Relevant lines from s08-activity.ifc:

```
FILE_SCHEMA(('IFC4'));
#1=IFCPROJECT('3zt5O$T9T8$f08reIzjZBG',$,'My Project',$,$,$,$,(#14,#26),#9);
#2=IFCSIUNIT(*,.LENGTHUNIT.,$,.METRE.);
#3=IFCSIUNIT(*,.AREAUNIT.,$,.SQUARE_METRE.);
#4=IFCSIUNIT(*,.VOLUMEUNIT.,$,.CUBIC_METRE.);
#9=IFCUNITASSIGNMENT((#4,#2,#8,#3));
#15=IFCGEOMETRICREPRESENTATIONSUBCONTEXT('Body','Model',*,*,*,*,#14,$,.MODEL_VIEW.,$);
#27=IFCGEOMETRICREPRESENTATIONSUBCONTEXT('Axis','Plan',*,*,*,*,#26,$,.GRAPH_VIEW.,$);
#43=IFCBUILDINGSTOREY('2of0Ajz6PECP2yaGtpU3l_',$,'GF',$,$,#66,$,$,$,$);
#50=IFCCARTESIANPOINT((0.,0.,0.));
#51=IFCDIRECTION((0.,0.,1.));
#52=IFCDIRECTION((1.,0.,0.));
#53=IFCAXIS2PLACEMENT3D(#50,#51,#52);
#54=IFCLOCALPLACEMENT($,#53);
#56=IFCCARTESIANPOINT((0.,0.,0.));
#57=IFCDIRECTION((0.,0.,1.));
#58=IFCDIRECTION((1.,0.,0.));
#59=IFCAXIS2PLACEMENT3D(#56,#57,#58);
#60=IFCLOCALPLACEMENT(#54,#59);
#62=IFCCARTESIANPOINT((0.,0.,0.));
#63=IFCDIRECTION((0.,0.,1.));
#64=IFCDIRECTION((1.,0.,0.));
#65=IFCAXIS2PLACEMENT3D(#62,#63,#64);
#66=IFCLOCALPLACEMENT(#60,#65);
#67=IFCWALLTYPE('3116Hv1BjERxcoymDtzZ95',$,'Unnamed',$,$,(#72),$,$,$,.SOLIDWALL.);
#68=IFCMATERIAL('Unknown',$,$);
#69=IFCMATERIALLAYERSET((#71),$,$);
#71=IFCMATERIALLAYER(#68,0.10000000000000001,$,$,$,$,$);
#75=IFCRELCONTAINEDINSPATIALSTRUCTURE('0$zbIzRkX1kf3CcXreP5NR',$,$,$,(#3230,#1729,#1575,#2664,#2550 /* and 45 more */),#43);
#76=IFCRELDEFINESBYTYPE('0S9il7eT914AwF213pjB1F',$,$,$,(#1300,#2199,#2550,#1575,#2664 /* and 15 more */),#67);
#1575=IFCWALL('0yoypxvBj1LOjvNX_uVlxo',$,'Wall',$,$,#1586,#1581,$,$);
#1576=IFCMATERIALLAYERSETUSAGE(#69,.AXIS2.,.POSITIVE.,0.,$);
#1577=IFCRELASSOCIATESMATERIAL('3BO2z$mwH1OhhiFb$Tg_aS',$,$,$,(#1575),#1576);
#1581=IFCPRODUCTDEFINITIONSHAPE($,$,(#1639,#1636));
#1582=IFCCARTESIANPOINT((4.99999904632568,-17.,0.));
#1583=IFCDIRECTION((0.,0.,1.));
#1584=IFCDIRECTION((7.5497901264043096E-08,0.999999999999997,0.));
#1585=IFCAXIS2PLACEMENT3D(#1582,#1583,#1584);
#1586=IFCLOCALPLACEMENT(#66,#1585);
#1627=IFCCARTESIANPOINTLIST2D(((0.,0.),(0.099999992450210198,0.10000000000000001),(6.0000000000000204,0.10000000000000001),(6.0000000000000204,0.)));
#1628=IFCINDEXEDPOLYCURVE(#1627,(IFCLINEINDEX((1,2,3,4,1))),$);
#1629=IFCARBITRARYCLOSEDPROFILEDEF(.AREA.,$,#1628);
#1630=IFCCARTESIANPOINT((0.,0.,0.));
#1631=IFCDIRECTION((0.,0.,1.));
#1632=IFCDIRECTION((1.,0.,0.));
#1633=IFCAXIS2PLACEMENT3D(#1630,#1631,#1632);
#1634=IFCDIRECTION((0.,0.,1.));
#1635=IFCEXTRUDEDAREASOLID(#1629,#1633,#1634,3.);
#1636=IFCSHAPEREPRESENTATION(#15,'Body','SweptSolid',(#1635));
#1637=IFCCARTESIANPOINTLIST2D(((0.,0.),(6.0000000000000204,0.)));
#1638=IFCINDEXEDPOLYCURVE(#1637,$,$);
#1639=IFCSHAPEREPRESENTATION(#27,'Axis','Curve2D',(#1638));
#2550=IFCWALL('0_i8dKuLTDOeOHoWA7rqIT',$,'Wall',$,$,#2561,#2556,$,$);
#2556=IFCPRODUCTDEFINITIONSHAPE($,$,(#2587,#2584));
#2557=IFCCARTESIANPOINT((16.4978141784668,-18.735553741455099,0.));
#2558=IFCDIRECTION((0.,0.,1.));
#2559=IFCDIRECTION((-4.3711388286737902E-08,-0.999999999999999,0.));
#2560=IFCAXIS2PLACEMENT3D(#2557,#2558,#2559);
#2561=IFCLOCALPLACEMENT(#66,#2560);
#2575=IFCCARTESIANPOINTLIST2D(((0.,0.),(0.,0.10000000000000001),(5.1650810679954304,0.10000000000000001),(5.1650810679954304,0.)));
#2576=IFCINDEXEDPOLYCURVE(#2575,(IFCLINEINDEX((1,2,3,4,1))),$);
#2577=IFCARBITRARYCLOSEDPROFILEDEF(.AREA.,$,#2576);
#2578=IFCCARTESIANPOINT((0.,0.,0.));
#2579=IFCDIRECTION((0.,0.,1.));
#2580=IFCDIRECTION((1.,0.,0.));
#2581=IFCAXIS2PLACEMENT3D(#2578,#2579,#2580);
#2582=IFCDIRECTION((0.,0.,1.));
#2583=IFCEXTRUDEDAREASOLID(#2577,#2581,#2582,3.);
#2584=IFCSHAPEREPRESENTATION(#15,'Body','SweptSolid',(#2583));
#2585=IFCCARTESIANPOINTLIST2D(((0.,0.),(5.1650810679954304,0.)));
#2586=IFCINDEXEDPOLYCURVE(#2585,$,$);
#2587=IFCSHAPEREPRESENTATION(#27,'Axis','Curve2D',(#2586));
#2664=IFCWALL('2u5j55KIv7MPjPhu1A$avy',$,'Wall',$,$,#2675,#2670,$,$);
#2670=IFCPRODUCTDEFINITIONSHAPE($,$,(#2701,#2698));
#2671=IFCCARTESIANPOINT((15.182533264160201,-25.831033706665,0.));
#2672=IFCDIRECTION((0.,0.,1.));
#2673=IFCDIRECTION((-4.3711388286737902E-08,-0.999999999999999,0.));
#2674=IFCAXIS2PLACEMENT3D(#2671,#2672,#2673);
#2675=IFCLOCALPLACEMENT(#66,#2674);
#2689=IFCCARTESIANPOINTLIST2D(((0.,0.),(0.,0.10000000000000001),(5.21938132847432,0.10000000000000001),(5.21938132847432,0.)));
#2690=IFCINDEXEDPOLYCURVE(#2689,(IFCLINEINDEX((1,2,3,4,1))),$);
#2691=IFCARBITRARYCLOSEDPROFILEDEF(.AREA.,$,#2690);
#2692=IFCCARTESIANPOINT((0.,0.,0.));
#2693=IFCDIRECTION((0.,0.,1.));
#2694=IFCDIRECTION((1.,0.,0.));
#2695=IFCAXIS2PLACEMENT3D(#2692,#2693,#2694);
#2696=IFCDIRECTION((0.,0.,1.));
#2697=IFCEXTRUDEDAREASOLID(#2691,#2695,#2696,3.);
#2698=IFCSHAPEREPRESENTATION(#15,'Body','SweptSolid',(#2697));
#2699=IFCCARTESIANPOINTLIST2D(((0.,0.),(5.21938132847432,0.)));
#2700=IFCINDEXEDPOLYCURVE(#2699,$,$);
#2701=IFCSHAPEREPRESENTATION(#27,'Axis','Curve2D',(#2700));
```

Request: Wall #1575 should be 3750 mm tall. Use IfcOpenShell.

```python
import ifcopenshell
import ifcopenshell.geom
import ifcopenshell.util.representation
import ifcopenshell.util.shape

model = ifcopenshell.open("s08-activity.ifc")
settings = ifcopenshell.geom.settings()


def volume(element):
    """Net volume in cubic metres, openings subtracted."""
    shape = ifcopenshell.geom.create_shape(settings, element)
    return ifcopenshell.util.shape.get_volume(shape.geometry)


wall = model.by_guid("0yoypxvBj1LOjvNX_uVlxo")
before = volume(wall)

body = ifcopenshell.util.representation.get_representation(wall, "Model", "Body")
solid = body.Items[0]
old_height = solid.Depth
solid.Depth = 3.75
after = volume(wall)

print(f"height {old_height:g} -> {solid.Depth:g}, volume {before:.3f} -> {after:.3f} m3")

model.write("s08-activity_rev.ifc")
```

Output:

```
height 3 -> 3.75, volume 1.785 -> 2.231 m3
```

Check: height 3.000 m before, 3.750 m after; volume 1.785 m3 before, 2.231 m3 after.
